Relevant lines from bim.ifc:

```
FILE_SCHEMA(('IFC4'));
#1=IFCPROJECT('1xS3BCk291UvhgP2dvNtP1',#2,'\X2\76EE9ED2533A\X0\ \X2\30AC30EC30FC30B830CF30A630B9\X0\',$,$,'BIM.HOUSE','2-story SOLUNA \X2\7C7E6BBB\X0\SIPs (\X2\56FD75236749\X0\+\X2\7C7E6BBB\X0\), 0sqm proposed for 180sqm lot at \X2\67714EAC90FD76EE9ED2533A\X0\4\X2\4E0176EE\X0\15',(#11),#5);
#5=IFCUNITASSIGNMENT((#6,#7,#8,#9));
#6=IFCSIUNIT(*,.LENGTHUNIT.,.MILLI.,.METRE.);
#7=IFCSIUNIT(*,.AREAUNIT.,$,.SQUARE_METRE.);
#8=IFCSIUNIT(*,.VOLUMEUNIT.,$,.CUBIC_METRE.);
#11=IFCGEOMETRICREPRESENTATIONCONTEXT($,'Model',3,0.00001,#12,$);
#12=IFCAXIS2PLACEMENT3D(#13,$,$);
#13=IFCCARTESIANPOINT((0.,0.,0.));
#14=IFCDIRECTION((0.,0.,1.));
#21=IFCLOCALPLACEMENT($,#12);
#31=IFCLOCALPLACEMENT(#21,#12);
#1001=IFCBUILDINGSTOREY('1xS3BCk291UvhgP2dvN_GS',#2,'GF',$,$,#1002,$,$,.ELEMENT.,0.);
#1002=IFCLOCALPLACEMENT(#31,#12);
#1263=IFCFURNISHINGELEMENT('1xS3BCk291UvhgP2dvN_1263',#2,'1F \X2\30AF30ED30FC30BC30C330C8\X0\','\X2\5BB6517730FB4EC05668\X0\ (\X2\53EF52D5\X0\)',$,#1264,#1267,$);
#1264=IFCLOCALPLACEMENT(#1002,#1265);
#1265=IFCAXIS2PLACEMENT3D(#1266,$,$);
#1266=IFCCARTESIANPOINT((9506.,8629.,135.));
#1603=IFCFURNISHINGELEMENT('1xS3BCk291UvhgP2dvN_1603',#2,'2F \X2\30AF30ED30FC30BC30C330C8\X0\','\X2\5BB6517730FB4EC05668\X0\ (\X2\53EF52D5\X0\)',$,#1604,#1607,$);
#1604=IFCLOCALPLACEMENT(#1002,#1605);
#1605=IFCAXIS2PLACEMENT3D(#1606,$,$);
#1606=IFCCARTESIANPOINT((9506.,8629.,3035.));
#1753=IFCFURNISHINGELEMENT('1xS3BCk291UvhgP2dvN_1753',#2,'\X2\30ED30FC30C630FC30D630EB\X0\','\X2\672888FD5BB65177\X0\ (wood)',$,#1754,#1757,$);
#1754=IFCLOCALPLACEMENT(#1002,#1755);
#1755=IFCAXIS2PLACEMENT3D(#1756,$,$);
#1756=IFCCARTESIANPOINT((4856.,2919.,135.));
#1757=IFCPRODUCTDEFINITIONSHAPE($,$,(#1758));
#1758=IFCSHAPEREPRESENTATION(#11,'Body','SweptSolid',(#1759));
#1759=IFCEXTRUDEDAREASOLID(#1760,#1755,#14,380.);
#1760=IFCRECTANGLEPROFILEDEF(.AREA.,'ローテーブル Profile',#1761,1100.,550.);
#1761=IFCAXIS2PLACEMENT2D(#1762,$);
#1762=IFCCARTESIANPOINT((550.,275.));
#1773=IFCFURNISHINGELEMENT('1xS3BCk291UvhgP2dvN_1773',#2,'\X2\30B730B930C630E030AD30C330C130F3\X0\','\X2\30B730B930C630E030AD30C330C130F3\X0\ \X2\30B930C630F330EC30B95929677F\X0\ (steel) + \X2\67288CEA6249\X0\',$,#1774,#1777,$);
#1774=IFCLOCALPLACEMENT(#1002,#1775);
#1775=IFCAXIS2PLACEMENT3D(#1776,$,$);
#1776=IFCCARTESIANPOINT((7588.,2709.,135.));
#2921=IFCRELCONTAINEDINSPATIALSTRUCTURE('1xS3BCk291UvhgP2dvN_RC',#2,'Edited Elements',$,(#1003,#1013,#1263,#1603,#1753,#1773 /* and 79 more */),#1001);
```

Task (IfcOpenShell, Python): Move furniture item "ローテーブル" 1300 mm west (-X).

```python
import ifcopenshell
import ifcopenshell.api.geometry
import ifcopenshell.util.placement

model = ifcopenshell.open("bim.ifc")

item = model.by_guid("1xS3BCk291UvhgP2dvN_1753")
matrix = ifcopenshell.util.placement.get_local_placement(item.ObjectPlacement)
matrix[0, 3] -= 1300.0
ifcopenshell.api.geometry.edit_object_placement(model, product=item, matrix=matrix, is_si=False)

print(ifcopenshell.util.placement.get_local_placement(item.ObjectPlacement).round(3) + 0.0)

model.write("bim_v2.ifc")
```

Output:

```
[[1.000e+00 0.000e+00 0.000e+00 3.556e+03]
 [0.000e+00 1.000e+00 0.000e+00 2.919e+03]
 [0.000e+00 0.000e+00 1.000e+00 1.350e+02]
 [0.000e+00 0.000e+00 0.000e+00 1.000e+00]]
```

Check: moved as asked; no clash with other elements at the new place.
